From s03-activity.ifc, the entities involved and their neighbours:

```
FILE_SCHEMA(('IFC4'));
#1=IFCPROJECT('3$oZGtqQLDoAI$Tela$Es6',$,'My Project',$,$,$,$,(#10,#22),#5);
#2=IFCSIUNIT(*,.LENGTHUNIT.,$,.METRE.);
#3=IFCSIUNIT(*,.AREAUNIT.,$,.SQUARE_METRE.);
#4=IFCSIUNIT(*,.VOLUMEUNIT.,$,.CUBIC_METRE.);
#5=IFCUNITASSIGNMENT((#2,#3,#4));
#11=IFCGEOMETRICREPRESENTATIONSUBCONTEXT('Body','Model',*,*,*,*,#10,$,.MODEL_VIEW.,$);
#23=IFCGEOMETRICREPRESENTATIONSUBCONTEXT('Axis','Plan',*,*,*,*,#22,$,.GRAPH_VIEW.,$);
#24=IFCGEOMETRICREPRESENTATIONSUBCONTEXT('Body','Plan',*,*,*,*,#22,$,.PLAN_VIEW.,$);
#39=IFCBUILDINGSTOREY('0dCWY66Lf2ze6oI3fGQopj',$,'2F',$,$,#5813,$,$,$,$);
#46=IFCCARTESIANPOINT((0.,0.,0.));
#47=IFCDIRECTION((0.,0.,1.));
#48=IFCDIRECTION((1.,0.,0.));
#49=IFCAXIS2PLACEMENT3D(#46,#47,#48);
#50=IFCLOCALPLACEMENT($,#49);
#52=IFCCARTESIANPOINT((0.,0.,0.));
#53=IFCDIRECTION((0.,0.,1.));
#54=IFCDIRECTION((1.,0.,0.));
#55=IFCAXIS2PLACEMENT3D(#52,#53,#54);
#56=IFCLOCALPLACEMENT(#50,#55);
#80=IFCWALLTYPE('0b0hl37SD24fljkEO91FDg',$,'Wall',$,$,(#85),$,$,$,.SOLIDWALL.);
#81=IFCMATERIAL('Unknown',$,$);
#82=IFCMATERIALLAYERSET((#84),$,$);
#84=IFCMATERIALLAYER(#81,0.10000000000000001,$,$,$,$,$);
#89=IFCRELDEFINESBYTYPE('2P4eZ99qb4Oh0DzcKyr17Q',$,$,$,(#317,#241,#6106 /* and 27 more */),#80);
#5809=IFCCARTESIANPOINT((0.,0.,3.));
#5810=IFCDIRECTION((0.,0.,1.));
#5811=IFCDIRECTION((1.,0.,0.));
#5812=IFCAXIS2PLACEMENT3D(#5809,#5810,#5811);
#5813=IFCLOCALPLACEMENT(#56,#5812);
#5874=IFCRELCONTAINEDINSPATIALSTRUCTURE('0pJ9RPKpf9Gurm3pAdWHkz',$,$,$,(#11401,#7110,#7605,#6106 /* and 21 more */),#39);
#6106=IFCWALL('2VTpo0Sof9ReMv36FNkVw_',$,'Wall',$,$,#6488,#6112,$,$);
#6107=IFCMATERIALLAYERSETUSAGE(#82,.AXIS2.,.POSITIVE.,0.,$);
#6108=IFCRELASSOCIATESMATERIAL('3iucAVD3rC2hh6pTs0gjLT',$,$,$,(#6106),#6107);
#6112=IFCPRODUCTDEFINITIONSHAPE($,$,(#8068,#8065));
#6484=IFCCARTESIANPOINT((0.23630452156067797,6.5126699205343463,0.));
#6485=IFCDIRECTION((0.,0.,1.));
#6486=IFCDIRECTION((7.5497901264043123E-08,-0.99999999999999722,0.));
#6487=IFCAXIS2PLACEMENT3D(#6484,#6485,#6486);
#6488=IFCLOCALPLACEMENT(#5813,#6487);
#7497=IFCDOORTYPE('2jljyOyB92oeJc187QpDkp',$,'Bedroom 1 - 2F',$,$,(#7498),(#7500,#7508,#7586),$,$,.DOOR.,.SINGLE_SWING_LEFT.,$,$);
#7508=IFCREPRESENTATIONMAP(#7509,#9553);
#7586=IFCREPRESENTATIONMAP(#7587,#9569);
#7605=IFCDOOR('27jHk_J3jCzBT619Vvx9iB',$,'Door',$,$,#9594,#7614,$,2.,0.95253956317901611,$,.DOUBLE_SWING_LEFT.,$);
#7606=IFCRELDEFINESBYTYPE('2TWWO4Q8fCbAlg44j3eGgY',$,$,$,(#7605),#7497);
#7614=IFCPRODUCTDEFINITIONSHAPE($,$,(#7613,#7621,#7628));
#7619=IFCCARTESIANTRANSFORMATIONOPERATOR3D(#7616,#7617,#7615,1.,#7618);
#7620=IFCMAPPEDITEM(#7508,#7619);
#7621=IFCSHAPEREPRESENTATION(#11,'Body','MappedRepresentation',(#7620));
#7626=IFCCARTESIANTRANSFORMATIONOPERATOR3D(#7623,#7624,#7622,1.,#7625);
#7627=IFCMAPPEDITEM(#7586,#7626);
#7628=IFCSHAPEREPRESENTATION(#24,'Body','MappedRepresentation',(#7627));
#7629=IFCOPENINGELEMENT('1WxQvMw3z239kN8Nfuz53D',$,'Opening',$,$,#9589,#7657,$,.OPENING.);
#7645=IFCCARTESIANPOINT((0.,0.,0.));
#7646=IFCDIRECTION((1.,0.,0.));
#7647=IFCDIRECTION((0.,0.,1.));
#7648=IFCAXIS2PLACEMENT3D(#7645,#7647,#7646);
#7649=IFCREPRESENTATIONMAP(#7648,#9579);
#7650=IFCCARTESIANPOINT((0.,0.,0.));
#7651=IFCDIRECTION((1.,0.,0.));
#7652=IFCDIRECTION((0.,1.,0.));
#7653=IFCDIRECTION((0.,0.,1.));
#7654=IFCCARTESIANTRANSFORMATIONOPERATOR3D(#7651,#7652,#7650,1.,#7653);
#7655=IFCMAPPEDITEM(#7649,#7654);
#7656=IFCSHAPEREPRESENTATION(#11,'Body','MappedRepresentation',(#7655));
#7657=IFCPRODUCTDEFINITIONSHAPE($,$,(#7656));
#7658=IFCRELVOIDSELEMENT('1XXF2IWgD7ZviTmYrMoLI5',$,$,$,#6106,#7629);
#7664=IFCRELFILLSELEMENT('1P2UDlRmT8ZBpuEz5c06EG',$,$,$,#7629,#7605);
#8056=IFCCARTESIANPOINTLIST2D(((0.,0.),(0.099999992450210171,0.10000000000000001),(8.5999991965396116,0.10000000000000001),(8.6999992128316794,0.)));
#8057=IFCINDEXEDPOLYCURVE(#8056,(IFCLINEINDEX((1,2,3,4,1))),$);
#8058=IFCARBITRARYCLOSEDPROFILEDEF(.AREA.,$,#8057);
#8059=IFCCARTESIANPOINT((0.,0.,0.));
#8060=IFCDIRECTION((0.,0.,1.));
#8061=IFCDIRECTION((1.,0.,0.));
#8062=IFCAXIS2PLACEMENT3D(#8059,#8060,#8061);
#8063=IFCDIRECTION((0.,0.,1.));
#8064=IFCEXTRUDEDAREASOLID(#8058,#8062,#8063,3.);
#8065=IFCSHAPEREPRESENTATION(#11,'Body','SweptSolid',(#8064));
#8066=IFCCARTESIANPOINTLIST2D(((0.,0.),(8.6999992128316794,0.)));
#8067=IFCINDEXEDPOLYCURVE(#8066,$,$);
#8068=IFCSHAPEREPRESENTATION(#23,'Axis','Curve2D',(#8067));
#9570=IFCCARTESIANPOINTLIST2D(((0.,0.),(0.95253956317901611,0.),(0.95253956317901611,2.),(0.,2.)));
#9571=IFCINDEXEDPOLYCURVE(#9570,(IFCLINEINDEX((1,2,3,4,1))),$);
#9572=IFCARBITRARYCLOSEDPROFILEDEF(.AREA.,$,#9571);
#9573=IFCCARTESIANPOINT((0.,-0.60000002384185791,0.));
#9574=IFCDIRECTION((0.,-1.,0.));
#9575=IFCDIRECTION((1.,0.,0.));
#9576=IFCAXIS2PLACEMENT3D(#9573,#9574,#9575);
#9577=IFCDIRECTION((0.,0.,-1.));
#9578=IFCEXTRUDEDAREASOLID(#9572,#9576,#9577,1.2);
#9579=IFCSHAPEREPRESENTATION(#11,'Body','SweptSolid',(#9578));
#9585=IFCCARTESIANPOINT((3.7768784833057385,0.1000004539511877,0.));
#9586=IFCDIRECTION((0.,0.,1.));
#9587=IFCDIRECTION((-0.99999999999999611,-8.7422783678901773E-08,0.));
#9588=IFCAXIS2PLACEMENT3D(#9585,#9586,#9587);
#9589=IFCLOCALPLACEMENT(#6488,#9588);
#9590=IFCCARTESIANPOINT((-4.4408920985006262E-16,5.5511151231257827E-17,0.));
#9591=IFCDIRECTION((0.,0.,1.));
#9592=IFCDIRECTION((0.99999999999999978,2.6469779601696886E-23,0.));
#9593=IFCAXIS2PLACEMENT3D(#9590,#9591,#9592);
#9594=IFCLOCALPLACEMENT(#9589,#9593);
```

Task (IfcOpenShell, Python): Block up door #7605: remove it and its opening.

```python
import ifcopenshell
import ifcopenshell.api.feature
import ifcopenshell.api.root
import ifcopenshell.geom
import ifcopenshell.util.shape

model = ifcopenshell.open("s03-activity.ifc")
settings = ifcopenshell.geom.settings()


def volume(element):
    """Net volume in cubic metres, openings subtracted."""
    shape = ifcopenshell.geom.create_shape(settings, element)
    return ifcopenshell.util.shape.get_volume(shape.geometry)


door = model.by_guid("27jHk_J3jCzBT619Vvx9iB")
opening = door.FillsVoids[0].RelatingOpeningElement
wall = opening.VoidsElements[0].RelatingBuildingElement
before = volume(wall)

ifcopenshell.api.root.remove_product(model, product=door)
ifcopenshell.api.feature.remove_feature(model, feature=opening)

after = volume(wall)

print(f"wall volume {before:.3f} -> {after:.3f} m3")

model.write("s03-activity_v2.ifc")
```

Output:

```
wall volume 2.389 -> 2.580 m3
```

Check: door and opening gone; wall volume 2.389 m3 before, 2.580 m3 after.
